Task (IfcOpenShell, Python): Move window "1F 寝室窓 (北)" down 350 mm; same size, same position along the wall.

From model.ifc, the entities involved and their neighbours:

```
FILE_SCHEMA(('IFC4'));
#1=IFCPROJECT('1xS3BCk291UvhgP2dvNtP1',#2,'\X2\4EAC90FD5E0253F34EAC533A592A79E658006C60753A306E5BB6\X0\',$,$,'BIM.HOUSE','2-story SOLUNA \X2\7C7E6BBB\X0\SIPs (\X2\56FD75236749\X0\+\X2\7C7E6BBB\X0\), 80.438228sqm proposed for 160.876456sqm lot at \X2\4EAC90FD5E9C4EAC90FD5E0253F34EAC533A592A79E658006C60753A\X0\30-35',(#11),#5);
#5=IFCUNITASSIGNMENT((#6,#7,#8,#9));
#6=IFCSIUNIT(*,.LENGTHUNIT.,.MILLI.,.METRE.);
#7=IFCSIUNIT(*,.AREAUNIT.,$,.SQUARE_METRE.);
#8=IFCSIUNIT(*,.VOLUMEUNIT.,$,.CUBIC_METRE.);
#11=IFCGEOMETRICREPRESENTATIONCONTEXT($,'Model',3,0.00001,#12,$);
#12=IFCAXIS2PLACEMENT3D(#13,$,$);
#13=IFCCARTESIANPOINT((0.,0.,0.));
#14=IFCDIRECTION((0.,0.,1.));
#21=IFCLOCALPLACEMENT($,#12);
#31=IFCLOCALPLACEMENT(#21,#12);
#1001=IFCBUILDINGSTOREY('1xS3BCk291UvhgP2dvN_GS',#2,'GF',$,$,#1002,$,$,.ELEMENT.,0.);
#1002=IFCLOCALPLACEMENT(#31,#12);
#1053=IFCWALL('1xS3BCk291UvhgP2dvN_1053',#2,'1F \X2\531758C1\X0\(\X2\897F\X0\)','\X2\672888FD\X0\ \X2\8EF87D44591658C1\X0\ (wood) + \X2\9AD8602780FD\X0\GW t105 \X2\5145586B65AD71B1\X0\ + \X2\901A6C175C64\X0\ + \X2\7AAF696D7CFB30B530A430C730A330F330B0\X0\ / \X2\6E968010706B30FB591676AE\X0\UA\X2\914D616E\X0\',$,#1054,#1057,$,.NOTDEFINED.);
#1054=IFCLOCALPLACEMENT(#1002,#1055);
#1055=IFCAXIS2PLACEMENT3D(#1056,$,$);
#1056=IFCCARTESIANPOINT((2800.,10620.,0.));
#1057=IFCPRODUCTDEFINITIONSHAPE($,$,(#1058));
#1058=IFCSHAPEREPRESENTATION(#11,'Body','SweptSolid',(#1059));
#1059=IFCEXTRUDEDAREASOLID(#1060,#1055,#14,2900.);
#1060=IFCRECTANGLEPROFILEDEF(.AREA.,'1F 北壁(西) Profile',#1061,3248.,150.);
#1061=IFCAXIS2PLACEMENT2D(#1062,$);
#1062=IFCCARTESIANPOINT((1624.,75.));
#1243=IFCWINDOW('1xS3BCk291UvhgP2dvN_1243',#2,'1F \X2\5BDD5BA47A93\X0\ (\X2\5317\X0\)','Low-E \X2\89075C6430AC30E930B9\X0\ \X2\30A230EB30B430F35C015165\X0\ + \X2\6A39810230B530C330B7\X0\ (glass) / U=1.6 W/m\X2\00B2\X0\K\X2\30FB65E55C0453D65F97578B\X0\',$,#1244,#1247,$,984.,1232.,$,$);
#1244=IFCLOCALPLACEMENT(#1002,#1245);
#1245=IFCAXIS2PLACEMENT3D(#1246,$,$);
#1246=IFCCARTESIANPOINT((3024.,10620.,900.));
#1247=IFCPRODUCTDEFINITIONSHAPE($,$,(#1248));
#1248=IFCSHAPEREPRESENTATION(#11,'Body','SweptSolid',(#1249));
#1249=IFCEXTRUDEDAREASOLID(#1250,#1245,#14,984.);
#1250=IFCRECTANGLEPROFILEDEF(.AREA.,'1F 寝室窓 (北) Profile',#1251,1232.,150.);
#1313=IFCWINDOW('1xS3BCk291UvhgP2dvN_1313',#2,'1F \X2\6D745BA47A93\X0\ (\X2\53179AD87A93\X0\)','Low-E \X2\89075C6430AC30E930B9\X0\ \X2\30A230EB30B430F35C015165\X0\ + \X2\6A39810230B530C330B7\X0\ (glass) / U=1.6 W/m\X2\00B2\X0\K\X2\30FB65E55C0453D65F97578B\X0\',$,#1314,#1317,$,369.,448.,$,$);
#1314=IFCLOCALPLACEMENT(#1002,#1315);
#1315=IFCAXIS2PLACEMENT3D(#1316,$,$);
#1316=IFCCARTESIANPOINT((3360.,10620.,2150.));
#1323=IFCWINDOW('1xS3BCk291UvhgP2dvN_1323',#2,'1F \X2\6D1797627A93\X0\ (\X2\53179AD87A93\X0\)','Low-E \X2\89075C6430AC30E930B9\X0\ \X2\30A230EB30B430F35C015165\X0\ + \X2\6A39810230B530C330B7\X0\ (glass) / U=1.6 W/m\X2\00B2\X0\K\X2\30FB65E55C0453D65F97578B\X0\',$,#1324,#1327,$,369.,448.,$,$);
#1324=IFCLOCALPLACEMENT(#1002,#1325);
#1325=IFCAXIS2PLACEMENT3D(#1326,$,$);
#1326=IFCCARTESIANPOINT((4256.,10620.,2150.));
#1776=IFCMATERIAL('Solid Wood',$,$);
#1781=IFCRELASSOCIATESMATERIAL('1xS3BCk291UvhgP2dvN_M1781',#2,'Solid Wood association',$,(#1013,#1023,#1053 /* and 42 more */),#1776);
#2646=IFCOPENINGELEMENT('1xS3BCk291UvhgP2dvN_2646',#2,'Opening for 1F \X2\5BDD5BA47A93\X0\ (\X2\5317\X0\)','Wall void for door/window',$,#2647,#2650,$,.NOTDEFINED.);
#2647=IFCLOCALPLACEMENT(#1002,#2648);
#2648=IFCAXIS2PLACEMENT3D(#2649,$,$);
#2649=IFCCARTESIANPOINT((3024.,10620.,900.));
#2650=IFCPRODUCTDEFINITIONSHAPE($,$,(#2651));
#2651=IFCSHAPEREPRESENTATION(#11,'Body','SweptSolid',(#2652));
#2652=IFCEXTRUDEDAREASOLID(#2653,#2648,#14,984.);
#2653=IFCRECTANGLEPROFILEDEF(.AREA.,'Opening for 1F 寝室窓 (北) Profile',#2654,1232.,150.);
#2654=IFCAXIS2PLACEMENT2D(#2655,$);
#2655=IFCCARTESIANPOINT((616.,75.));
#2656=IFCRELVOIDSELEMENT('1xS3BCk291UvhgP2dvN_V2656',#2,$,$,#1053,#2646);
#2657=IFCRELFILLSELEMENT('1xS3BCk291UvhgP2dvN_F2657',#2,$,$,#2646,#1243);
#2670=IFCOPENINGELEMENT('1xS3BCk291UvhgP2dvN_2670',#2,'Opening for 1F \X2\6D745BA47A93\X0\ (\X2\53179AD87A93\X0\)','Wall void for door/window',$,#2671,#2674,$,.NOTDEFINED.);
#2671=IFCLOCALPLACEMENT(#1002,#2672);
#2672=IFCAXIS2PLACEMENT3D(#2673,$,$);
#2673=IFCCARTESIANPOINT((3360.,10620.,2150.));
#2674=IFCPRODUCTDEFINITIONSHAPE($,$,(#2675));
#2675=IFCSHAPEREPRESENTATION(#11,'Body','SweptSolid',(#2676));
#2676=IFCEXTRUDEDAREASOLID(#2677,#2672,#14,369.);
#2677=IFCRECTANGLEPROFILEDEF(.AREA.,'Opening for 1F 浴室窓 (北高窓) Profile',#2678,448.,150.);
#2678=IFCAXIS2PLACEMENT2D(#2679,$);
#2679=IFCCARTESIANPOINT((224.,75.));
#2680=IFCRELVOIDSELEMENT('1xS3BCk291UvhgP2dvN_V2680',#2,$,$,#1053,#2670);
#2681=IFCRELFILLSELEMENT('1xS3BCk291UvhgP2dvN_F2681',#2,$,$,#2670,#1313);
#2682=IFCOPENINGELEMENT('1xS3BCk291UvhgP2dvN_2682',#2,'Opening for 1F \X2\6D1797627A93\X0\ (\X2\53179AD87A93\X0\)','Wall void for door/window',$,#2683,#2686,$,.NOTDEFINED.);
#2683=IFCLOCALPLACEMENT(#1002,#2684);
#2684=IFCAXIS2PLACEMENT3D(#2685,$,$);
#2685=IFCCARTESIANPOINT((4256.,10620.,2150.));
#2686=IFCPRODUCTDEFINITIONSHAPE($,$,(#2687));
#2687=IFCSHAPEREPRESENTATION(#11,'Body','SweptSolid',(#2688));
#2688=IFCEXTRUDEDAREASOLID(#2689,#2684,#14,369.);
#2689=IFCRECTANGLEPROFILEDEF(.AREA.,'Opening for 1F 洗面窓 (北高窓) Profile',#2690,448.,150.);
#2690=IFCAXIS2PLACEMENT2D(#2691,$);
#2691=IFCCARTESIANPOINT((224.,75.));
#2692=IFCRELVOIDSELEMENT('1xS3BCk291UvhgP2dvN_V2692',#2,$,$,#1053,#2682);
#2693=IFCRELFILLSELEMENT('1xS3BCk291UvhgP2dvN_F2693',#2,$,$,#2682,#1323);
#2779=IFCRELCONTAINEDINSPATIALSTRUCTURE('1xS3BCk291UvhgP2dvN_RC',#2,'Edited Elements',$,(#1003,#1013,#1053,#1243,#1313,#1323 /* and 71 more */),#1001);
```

```python
import numpy as np
import ifcopenshell
import ifcopenshell.api.geometry
import ifcopenshell.util.placement
import ifcopenshell.util.unit

model = ifcopenshell.open("model.ifc")
unit_scale = ifcopenshell.util.unit.calculate_unit_scale(model)

window = model.by_guid("1xS3BCk291UvhgP2dvN_1243")
opening = window.FillsVoids[0].RelatingOpeningElement
dz = -0.35 / unit_scale

shift = np.array([0.0, 0.0, dz])
# The window is not placed relative to its opening, so move both.
for product in (opening, window):
    matrix = ifcopenshell.util.placement.get_local_placement(product.ObjectPlacement)
    matrix[:3, 3] += shift
    ifcopenshell.api.geometry.edit_object_placement(model, product=product, matrix=matrix, is_si=False)

print(f"moved by {dz * unit_scale:+.3f} m")

model.write("model_v2.ifc")
```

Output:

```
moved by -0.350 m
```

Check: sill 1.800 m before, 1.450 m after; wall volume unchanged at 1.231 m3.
